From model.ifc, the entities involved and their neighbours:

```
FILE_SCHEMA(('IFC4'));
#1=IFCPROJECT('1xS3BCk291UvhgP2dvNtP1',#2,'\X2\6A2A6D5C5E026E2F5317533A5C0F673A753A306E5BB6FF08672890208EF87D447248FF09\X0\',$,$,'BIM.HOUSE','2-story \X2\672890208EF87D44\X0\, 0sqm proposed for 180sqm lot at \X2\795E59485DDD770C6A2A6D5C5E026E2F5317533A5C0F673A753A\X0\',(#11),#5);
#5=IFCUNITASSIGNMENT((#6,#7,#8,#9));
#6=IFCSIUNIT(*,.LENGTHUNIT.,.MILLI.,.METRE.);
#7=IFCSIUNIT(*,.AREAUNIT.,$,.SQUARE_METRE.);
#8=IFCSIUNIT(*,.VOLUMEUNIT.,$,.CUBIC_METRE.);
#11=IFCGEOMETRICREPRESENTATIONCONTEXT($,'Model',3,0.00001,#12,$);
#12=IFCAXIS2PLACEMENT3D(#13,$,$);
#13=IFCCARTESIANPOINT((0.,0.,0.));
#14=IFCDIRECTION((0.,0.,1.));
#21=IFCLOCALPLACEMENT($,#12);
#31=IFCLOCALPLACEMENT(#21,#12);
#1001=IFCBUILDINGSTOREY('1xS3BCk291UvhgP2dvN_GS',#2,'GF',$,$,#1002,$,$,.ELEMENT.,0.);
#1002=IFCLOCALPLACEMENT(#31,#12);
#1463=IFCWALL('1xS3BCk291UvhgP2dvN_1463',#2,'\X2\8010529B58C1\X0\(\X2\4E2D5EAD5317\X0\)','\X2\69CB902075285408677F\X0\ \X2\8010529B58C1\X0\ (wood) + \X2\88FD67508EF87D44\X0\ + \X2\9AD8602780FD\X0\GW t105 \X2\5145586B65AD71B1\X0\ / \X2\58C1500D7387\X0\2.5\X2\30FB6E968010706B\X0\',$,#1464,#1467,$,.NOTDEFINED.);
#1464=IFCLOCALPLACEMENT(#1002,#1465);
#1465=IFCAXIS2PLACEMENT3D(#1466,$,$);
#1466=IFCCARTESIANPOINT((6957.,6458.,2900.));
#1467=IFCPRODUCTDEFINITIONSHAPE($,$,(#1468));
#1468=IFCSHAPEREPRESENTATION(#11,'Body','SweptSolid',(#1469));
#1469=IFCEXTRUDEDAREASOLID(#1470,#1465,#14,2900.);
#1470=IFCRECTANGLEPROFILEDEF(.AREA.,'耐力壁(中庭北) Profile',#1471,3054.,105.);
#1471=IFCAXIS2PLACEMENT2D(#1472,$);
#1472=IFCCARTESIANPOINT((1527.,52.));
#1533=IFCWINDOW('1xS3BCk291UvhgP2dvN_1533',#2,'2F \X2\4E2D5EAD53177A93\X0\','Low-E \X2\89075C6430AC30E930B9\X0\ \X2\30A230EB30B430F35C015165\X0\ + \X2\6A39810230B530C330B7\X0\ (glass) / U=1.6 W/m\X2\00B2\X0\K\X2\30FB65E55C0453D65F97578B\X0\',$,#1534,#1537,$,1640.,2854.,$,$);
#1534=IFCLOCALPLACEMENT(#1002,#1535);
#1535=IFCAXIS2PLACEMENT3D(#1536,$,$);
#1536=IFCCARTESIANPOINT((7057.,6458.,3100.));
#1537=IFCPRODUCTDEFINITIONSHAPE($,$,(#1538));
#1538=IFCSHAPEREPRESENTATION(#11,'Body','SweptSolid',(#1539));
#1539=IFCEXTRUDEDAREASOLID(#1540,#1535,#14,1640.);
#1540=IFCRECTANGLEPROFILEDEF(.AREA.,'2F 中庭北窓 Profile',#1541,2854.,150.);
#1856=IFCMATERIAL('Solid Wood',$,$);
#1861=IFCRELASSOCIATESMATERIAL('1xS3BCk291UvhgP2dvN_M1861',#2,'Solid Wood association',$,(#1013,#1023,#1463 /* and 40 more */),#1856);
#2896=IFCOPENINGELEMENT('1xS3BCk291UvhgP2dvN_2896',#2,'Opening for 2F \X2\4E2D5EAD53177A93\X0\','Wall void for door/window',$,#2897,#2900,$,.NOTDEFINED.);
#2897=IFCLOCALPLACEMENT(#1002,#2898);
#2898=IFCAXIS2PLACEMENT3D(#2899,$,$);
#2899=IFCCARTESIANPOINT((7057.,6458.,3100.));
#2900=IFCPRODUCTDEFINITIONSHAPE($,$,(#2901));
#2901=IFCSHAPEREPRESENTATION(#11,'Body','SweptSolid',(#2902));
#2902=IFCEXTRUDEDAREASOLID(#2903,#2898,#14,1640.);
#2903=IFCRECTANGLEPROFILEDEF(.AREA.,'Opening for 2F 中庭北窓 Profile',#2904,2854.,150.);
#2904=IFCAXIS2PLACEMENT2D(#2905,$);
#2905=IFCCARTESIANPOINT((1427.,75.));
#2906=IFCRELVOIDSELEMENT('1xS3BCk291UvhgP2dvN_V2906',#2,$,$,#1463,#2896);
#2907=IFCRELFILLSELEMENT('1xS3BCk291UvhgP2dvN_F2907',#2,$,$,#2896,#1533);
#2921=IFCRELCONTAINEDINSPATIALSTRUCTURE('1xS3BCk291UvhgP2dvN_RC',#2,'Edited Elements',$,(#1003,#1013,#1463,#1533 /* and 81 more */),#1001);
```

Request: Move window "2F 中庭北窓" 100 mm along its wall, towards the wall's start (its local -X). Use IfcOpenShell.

```python
import ifcopenshell
import ifcopenshell.api.geometry
import ifcopenshell.util.placement
import ifcopenshell.util.unit

model = ifcopenshell.open("model.ifc")
unit_scale = ifcopenshell.util.unit.calculate_unit_scale(model)

window = model.by_guid("1xS3BCk291UvhgP2dvN_1533")
opening = window.FillsVoids[0].RelatingOpeningElement
wall = opening.VoidsElements[0].RelatingBuildingElement

wall_matrix = ifcopenshell.util.placement.get_local_placement(wall.ObjectPlacement)
shift = wall_matrix[:3, 0] * -0.1 / unit_scale
before = ifcopenshell.util.placement.get_local_placement(window.ObjectPlacement)[:3, 3].copy()

# The window is not placed relative to its opening, so move both.
for product in (opening, window):
    matrix = ifcopenshell.util.placement.get_local_placement(product.ObjectPlacement)
    matrix[:3, 3] += shift
    ifcopenshell.api.geometry.edit_object_placement(model, product=product, matrix=matrix, is_si=False)

after = ifcopenshell.util.placement.get_local_placement(window.ObjectPlacement)[:3, 3]
print("window moved by", (after - before).round(3) + 0.0)

model.write("model-out.ifc")
```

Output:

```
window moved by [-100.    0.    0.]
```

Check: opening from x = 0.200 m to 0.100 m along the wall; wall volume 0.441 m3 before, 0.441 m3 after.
